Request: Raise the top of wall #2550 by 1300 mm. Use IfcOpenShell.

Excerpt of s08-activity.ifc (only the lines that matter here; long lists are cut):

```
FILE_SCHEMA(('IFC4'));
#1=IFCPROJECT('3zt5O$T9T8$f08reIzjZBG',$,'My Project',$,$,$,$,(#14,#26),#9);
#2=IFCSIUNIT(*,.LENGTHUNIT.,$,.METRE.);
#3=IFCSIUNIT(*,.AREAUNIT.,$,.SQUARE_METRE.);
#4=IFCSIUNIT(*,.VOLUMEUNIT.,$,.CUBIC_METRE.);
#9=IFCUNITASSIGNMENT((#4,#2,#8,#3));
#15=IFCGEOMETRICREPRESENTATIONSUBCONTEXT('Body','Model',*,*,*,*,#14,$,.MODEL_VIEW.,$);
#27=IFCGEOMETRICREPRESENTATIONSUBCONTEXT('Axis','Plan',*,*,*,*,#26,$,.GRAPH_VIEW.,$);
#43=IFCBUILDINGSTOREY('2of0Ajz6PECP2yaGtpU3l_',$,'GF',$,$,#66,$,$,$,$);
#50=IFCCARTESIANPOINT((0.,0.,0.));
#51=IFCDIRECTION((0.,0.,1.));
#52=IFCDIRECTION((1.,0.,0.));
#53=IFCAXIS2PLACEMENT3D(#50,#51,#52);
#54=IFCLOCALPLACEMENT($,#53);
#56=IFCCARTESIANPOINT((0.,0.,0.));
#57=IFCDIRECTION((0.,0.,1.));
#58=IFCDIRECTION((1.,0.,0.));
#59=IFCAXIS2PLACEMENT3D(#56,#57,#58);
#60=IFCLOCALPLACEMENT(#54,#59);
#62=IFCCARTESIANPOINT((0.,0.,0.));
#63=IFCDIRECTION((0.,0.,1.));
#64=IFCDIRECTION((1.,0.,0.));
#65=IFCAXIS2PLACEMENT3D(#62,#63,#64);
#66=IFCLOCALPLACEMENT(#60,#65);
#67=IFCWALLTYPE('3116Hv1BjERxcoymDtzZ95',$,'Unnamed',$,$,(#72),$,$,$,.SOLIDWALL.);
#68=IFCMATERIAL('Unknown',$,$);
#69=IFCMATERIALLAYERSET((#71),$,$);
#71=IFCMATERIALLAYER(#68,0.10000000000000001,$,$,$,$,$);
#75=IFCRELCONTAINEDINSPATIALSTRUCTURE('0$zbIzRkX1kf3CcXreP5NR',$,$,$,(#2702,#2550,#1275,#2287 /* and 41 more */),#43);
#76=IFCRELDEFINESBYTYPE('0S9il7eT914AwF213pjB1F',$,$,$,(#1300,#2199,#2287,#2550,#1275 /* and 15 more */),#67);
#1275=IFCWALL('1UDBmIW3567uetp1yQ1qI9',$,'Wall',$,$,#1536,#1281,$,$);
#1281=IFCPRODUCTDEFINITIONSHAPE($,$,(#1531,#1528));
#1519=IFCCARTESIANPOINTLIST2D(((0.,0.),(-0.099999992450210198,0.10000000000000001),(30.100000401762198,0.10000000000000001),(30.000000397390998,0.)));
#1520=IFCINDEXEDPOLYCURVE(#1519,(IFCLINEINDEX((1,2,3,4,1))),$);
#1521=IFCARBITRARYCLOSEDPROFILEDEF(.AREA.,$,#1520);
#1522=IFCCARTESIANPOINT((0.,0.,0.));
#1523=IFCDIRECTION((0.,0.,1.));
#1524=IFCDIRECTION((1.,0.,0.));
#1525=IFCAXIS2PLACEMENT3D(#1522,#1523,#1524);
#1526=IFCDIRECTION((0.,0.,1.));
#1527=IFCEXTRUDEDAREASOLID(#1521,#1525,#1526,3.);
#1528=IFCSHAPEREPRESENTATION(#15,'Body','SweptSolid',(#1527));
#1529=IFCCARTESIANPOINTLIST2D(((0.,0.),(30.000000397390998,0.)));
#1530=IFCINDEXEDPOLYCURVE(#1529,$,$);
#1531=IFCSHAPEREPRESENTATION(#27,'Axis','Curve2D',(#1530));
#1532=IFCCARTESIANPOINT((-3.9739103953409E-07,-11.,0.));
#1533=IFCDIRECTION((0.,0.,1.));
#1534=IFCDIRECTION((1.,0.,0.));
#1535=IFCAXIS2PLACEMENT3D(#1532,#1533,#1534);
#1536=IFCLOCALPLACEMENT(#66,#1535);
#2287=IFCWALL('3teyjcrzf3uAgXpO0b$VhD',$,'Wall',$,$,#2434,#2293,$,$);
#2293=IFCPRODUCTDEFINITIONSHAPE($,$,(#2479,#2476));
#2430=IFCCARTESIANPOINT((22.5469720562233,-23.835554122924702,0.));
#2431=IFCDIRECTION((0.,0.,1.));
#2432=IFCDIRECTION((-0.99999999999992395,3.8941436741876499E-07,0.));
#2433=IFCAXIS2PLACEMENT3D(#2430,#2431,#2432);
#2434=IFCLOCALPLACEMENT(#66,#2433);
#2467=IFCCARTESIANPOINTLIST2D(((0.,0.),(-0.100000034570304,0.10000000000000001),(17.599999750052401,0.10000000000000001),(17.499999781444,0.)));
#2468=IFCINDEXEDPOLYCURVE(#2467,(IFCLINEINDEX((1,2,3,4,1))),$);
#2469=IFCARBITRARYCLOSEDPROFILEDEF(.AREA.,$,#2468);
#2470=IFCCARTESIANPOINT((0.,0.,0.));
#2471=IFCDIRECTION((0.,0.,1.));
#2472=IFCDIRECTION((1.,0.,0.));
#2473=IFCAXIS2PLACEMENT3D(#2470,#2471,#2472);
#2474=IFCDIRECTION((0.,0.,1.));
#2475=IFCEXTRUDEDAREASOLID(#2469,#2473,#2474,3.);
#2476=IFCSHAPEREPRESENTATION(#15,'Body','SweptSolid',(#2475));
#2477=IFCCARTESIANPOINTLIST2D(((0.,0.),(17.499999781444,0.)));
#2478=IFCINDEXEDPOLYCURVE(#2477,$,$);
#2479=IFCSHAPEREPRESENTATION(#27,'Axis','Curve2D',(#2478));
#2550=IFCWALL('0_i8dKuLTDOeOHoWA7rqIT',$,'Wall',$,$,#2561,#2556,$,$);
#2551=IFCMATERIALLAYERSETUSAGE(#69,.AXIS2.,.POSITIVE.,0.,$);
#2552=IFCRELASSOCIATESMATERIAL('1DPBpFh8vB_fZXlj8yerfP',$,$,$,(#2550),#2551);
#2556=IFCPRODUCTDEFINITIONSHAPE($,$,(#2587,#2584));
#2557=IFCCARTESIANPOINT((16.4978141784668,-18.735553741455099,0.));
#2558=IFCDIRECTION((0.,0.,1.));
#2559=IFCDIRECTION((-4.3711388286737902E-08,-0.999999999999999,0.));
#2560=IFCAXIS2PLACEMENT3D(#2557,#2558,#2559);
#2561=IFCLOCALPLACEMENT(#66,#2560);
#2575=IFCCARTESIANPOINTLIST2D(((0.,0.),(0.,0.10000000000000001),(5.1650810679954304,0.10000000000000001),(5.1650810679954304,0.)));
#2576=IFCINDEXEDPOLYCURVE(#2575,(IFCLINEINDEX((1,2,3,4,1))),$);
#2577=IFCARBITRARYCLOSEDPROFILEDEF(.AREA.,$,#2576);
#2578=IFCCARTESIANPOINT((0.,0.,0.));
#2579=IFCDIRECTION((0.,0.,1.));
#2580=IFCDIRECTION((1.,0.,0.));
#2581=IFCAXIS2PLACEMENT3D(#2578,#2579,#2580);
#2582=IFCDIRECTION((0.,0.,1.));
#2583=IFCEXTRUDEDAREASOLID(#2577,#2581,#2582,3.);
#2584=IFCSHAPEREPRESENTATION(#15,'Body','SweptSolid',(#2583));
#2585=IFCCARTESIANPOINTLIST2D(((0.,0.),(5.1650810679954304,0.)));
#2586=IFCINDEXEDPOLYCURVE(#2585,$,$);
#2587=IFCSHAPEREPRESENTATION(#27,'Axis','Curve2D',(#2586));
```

```python
import ifcopenshell
import ifcopenshell.geom
import ifcopenshell.util.representation
import ifcopenshell.util.shape

model = ifcopenshell.open("s08-activity.ifc")
settings = ifcopenshell.geom.settings()


def volume(element):
    """Net volume in cubic metres, openings subtracted."""
    shape = ifcopenshell.geom.create_shape(settings, element)
    return ifcopenshell.util.shape.get_volume(shape.geometry)


wall = model.by_guid("0_i8dKuLTDOeOHoWA7rqIT")
before = volume(wall)

body = ifcopenshell.util.representation.get_representation(wall, "Model", "Body")
solid = body.Items[0]
old_height = solid.Depth
solid.Depth += 1.3
after = volume(wall)

print(f"height {old_height:g} -> {solid.Depth:g}, volume {before:.3f} -> {after:.3f} m3")

model.write("s08-activity_edited.ifc")
```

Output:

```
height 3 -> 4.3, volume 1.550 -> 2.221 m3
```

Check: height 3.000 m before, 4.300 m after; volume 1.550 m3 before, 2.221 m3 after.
